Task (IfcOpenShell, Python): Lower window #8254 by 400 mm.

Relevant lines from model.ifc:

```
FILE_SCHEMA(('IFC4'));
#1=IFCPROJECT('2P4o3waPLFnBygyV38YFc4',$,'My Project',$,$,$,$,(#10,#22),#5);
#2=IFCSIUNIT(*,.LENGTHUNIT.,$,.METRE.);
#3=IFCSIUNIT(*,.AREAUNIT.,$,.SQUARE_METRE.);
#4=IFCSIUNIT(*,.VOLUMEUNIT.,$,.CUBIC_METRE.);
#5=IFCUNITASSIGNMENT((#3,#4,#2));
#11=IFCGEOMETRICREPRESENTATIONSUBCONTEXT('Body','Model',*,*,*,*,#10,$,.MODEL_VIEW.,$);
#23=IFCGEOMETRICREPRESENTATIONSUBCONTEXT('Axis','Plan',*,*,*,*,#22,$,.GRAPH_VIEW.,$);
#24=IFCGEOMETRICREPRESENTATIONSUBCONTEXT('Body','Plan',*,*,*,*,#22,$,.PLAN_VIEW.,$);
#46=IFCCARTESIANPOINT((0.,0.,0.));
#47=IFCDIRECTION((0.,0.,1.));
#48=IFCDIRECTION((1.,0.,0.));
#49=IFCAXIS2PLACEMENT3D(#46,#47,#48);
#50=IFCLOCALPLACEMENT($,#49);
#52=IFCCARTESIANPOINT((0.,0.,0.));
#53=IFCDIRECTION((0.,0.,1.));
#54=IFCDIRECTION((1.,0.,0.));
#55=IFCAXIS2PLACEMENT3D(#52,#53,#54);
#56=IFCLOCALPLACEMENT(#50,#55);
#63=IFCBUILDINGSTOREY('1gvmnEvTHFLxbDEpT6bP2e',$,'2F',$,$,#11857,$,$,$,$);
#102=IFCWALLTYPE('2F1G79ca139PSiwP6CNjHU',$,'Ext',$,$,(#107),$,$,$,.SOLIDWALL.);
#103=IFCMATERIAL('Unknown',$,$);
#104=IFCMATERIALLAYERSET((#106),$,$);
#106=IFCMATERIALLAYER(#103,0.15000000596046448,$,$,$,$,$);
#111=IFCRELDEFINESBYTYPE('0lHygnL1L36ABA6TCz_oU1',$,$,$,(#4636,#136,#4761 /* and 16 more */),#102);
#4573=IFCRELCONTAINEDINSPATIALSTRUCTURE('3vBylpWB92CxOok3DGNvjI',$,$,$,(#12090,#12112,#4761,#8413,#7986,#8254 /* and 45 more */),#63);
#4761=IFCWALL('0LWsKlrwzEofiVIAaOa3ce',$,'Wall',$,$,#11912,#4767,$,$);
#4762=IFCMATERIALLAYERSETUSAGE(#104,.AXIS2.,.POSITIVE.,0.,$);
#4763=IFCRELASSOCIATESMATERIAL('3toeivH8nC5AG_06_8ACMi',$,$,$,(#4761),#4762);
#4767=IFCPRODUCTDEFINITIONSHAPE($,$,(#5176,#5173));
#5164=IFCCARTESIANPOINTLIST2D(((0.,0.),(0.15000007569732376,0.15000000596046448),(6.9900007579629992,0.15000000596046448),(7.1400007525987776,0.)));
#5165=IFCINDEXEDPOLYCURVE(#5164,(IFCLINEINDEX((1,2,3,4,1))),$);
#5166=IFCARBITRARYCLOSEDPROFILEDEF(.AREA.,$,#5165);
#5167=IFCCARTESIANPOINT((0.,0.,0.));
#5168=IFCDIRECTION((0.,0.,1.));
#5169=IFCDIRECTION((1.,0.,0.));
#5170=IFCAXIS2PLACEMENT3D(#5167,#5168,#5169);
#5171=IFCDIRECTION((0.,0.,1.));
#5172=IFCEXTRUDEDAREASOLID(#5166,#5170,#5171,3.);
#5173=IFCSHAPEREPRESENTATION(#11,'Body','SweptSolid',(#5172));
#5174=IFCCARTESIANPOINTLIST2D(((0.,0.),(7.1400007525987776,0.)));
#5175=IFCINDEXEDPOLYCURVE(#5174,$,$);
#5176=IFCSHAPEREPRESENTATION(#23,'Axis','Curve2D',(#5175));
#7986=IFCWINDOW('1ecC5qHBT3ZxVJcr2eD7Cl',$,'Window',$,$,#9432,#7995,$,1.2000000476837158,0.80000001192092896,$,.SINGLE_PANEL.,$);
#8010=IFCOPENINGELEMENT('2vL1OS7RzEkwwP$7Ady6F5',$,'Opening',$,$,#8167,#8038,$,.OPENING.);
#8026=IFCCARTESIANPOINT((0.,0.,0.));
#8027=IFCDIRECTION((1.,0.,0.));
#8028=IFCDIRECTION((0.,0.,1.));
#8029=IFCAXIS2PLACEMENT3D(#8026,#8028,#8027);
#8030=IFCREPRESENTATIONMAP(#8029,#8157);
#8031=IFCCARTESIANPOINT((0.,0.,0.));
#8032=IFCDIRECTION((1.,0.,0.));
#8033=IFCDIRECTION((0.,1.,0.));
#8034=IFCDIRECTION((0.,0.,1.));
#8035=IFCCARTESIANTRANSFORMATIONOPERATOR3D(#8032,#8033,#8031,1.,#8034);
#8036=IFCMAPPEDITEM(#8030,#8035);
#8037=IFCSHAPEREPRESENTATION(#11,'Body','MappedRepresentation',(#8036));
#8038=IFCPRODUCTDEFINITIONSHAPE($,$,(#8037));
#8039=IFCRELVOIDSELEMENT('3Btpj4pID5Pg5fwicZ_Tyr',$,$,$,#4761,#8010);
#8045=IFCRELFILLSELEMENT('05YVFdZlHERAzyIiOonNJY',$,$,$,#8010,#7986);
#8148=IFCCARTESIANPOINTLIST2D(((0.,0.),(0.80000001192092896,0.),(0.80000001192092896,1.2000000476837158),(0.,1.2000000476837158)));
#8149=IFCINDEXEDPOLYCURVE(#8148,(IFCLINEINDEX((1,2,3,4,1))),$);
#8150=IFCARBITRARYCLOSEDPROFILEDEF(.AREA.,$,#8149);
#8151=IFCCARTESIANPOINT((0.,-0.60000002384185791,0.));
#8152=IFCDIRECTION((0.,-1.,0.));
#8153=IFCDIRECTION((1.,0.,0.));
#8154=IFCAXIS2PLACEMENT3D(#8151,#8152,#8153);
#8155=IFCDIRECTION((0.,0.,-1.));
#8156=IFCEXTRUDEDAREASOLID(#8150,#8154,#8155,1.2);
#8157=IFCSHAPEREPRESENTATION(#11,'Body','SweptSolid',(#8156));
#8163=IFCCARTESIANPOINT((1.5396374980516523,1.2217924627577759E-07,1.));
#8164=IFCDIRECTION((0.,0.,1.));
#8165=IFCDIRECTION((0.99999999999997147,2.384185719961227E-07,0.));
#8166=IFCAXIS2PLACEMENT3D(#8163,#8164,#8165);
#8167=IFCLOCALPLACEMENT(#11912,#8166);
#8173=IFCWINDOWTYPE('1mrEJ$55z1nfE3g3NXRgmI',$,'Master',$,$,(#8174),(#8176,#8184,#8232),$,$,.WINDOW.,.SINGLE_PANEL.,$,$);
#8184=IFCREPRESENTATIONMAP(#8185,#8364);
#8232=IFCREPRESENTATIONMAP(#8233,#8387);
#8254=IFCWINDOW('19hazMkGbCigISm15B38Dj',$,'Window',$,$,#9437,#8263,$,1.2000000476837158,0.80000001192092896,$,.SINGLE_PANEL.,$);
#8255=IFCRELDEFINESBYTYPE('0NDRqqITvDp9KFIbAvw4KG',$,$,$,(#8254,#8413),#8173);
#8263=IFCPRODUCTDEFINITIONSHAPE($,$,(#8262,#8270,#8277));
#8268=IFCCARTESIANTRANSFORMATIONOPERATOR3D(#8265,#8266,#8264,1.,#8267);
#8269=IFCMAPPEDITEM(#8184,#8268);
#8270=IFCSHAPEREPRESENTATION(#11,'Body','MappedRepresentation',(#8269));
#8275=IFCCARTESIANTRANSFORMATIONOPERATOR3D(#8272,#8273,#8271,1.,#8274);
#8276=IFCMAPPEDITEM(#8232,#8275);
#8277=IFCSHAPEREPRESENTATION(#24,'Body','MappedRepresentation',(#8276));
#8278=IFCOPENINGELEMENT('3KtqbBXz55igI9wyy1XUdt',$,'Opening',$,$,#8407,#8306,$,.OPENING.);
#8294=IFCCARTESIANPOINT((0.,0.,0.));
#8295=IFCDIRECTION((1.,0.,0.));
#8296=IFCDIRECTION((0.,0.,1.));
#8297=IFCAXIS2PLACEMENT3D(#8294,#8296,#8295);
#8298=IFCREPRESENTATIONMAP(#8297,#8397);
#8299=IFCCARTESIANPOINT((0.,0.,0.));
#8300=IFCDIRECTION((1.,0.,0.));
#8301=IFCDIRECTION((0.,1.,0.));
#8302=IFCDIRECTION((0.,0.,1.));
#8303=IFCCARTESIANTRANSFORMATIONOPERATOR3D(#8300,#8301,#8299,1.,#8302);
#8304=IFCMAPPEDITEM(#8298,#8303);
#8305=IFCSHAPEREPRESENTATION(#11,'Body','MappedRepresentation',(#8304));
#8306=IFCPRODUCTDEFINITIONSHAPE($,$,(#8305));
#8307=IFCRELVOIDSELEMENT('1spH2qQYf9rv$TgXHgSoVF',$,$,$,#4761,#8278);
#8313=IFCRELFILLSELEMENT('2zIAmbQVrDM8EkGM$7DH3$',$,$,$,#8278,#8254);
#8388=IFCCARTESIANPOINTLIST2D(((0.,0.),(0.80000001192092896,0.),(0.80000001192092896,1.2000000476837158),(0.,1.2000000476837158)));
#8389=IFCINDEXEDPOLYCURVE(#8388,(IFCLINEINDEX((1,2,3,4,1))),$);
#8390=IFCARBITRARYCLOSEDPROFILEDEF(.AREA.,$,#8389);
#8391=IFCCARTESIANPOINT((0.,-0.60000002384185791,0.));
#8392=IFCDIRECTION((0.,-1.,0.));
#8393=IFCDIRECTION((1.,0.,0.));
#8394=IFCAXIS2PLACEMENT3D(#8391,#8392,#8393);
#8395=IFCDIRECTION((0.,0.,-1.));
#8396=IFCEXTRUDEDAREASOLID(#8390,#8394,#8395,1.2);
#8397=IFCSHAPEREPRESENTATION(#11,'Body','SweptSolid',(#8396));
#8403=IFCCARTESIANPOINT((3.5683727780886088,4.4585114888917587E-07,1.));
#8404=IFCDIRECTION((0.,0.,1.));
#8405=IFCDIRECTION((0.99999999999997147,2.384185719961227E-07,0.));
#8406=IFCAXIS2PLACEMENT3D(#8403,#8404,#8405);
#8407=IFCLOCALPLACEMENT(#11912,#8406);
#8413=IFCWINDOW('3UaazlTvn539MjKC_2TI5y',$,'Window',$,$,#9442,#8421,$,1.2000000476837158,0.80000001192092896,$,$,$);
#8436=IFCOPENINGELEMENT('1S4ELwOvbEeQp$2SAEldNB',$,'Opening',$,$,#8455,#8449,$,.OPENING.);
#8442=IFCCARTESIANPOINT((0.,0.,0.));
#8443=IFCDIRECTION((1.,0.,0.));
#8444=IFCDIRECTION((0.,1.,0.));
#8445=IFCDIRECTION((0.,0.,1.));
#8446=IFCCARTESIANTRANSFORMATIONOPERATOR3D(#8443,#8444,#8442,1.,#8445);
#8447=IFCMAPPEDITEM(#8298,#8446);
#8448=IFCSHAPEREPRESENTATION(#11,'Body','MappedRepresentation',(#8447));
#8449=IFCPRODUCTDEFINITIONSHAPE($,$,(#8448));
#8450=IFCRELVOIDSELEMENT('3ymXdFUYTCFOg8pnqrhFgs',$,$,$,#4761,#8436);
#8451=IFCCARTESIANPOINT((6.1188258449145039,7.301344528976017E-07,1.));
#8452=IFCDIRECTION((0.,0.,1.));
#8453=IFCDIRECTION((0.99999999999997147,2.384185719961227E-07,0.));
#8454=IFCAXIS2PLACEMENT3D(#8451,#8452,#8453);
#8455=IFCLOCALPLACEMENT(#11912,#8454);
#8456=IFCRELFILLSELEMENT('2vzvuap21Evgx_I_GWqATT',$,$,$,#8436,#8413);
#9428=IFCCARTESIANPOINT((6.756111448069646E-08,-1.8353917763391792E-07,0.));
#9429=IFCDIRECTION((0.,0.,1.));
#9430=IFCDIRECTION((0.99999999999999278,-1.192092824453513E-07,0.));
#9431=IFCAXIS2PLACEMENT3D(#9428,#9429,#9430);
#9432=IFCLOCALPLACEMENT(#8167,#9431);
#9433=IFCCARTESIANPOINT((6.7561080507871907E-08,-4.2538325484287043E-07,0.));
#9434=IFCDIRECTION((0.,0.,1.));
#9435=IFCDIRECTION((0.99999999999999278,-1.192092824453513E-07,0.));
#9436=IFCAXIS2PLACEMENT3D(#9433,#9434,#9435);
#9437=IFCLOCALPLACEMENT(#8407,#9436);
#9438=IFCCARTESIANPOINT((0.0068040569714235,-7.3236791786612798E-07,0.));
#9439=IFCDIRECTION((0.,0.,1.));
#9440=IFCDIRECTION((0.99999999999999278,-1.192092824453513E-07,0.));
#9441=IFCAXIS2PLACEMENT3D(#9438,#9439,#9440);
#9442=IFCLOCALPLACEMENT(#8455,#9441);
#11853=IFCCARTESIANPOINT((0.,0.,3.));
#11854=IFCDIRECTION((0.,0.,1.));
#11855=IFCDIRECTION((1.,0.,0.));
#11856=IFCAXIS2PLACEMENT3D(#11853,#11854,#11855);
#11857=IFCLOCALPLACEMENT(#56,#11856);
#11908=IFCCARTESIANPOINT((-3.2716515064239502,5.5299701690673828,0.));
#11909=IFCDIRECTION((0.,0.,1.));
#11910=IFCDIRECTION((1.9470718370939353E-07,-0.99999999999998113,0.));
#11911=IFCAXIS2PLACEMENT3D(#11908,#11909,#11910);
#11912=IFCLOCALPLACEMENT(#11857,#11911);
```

```python
import numpy as np
import ifcopenshell
import ifcopenshell.api.geometry
import ifcopenshell.util.placement
import ifcopenshell.util.unit

model = ifcopenshell.open("model.ifc")
unit_scale = ifcopenshell.util.unit.calculate_unit_scale(model)

window = model.by_id(8254)
opening = window.FillsVoids[0].RelatingOpeningElement
dz = -0.4

shift = np.array([0.0, 0.0, dz])
# The window is placed relative to its opening, so it follows when the opening moves.
matrix = ifcopenshell.util.placement.get_local_placement(opening.ObjectPlacement)
matrix[:3, 3] += shift
ifcopenshell.api.geometry.edit_object_placement(
    model, product=opening, matrix=matrix, is_si=False, should_transform_children=True
)

print(f"moved by {dz * unit_scale:+.3f} m")

model.write("model_v2.ifc")
```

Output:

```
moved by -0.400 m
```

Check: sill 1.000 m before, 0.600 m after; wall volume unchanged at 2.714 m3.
